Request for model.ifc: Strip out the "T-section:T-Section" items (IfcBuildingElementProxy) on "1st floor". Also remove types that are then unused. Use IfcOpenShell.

First a look at what the model holds.

```python
import ifcopenshell
import ifcopenshell.util.element

model = ifcopenshell.open("model.ifc")
print(model.schema)
storey = next(s for s in model.by_type("IfcBuildingStorey") if s.Name == "1st floor")
proxies = [e for e in ifcopenshell.util.element.get_decomposition(storey) if e.is_a("IfcBuildingElementProxy")]
seen = {}
for e in proxies:
    element_type = ifcopenshell.util.element.get_type(e)
    name = element_type.Name if element_type not in (None, e) else None
    seen[name] = seen.get(name, 0) + 1
for name, count in sorted(seen.items(), key=str):
    print(count, "x", name)
```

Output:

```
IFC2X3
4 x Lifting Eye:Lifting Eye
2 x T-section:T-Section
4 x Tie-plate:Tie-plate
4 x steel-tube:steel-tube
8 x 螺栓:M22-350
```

```python
import ifcopenshell
import ifcopenshell.api.root
import ifcopenshell.util.element

model = ifcopenshell.open("model.ifc")

storey = next(s for s in model.by_type("IfcBuildingStorey") if s.Name == "1st floor")
proxies = [e for e in ifcopenshell.util.element.get_decomposition(storey) if e.is_a("IfcBuildingElementProxy")]
targets = [e for e in proxies if (t := ifcopenshell.util.element.get_type(e)) not in (None, e) and t.Name == "T-section:T-Section"]
types = {ifcopenshell.util.element.get_type(e) for e in targets} - {None, *targets}

for e in targets:
    ifcopenshell.api.root.remove_product(model, product=e)
print(len(targets), "removed")

unused = [t for t in types if not ifcopenshell.util.element.get_types(t)]
for t in unused:
    ifcopenshell.api.root.remove_product(model, product=t)
print(len(unused), "unused types removed")

model.write("model-out.ifc")
```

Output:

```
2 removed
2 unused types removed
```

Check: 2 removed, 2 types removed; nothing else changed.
